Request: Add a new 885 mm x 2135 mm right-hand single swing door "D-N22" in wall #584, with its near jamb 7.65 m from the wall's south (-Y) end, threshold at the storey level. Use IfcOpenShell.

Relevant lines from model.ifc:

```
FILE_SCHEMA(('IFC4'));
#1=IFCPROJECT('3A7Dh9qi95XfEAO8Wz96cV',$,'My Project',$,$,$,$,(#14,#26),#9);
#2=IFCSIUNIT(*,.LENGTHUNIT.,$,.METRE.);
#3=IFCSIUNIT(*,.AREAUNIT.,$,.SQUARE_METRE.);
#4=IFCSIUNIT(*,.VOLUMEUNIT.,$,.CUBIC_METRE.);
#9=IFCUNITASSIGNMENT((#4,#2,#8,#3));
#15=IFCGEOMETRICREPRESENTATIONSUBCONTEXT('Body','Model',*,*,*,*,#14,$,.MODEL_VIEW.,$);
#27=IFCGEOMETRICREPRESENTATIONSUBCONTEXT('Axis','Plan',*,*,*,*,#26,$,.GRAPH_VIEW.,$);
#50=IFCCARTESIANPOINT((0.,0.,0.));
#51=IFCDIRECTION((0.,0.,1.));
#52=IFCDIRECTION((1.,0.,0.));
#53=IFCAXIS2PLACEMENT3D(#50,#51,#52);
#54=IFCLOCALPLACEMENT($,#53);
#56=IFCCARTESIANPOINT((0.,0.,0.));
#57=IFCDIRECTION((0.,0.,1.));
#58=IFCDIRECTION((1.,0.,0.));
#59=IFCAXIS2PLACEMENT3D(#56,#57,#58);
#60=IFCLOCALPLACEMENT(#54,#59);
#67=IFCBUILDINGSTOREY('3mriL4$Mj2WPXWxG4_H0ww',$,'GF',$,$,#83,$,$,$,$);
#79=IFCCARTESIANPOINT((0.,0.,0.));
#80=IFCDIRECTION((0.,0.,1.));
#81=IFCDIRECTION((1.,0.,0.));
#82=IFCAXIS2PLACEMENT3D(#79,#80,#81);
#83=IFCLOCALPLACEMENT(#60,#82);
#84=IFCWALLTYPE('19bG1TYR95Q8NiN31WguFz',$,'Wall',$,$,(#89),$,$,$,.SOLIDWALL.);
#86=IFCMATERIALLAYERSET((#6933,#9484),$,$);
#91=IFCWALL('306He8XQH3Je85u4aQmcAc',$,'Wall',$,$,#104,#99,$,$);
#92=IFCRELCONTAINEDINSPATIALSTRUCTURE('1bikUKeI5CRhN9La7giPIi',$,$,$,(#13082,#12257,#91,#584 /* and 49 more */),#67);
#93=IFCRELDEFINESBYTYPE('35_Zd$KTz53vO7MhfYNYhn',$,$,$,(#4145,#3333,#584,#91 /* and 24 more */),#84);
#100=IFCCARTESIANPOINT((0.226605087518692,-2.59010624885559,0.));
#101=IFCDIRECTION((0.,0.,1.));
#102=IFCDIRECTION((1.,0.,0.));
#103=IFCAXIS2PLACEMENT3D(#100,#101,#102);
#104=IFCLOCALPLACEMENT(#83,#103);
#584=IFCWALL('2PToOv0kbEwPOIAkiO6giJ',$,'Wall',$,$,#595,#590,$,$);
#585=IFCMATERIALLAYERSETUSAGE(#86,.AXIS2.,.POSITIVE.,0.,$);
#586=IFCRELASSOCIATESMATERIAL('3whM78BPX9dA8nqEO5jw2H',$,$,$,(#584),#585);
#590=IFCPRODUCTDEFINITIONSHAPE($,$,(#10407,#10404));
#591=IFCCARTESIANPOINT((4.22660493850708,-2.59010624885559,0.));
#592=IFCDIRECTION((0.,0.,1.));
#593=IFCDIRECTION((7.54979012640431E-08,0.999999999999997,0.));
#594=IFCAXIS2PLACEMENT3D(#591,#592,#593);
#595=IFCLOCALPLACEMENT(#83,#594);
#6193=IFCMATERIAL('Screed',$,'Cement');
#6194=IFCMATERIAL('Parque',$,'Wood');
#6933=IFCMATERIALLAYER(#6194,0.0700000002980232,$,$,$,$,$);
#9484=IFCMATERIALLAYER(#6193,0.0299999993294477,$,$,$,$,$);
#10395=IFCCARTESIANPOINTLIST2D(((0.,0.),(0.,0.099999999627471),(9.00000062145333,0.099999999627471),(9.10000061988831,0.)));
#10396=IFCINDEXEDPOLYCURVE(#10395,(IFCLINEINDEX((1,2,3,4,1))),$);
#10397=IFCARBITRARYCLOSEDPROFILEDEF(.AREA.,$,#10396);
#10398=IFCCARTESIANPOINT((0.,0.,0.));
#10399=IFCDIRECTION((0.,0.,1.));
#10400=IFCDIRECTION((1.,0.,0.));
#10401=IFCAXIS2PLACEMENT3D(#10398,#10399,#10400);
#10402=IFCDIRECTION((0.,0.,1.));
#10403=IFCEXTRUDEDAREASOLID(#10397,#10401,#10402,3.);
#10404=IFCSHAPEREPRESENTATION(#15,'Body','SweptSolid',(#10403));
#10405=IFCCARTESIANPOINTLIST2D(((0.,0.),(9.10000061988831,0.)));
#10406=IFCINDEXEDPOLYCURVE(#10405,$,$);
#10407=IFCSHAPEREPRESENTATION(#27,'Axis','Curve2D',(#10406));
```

```python
import numpy as np
import ifcopenshell
import ifcopenshell.api.feature
import ifcopenshell.api.geometry
import ifcopenshell.api.root
import ifcopenshell.api.spatial
import ifcopenshell.geom
import ifcopenshell.util.element
import ifcopenshell.util.placement
import ifcopenshell.util.representation
import ifcopenshell.util.shape
import ifcopenshell.util.unit

model = ifcopenshell.open("model.ifc")
unit_scale = ifcopenshell.util.unit.calculate_unit_scale(model)
settings = ifcopenshell.geom.settings()


def volume(element):
    """Net volume in cubic metres, openings subtracted."""
    shape = ifcopenshell.geom.create_shape(settings, element)
    return ifcopenshell.util.shape.get_volume(shape.geometry)


wall = model.by_guid("2PToOv0kbEwPOIAkiO6giJ")
storey = ifcopenshell.util.element.get_container(wall, ifc_class="IfcBuildingStorey")
context = ifcopenshell.util.representation.get_context(model, "Model", "Body", "MODEL_VIEW")
before = volume(wall)

width, height, from_end, sill = 0.885, 2.135, 7.65, 0.0  # metres

# The wall runs along its own X axis, and the end named is its -X end.
wall_shape = ifcopenshell.geom.create_shape(settings, wall)
x, y, z = ifcopenshell.util.shape.get_vertices(wall_shape.geometry).T
start = x.min() + from_end
face, thickness = float(y.min()), float(y.max() - y.min())
wall_matrix = ifcopenshell.util.placement.get_local_placement(wall.ObjectPlacement)
level = ifcopenshell.util.placement.get_local_placement(storey.ObjectPlacement)[2, 3]


def in_wall(x, y):
    """Placement at x, y metres in the wall's axes, at sill height."""
    matrix = wall_matrix.copy()
    matrix[:, 3] = wall_matrix @ np.array([x / unit_scale, y / unit_scale, 0.0, 1.0])
    matrix[2, 3] = level + sill / unit_scale
    return matrix


# Opening: a box that overshoots both wall faces by 50 mm.
opening = ifcopenshell.api.root.create_entity(model, ifc_class="IfcOpeningElement", predefined_type="OPENING")
box = ifcopenshell.api.geometry.add_wall_representation(
    model, context=context, length=width, height=height, thickness=thickness + 0.1
)
ifcopenshell.api.geometry.assign_representation(model, product=opening, representation=box)
ifcopenshell.api.geometry.edit_object_placement(model, product=opening, matrix=in_wall(start, face - 0.05), is_si=False)
ifcopenshell.api.feature.add_feature(model, feature=opening, element=wall)

door = ifcopenshell.api.root.create_entity(model, ifc_class="IfcDoor", name="D-N22", predefined_type="DOOR")
door.OverallWidth, door.OverallHeight = width / unit_scale, height / unit_scale
door.OperationType = "SINGLE_SWING_RIGHT"
body = ifcopenshell.api.geometry.add_door_representation(
    model,
    context=context,
    overall_width=door.OverallWidth,
    overall_height=door.OverallHeight,
    operation_type="SINGLE_SWING_RIGHT",
    lining_properties={"LiningDepth": thickness / unit_scale, "ThresholdDepth": thickness / unit_scale},
)
ifcopenshell.api.geometry.assign_representation(model, product=door, representation=body)
ifcopenshell.api.spatial.assign_container(model, products=[door], relating_structure=storey)
ifcopenshell.api.feature.add_filling(model, opening=opening, element=door)

# The lining spans the wall, so the door starts at the wall face.
ifcopenshell.api.geometry.edit_object_placement(model, product=door, matrix=in_wall(start, face), is_si=False)

after = volume(wall)

print(f"wall volume {before:.3f} -> {after:.3f} m3")

model.write("model_v2.ifc")
```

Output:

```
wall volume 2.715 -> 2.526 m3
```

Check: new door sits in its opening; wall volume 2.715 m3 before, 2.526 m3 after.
